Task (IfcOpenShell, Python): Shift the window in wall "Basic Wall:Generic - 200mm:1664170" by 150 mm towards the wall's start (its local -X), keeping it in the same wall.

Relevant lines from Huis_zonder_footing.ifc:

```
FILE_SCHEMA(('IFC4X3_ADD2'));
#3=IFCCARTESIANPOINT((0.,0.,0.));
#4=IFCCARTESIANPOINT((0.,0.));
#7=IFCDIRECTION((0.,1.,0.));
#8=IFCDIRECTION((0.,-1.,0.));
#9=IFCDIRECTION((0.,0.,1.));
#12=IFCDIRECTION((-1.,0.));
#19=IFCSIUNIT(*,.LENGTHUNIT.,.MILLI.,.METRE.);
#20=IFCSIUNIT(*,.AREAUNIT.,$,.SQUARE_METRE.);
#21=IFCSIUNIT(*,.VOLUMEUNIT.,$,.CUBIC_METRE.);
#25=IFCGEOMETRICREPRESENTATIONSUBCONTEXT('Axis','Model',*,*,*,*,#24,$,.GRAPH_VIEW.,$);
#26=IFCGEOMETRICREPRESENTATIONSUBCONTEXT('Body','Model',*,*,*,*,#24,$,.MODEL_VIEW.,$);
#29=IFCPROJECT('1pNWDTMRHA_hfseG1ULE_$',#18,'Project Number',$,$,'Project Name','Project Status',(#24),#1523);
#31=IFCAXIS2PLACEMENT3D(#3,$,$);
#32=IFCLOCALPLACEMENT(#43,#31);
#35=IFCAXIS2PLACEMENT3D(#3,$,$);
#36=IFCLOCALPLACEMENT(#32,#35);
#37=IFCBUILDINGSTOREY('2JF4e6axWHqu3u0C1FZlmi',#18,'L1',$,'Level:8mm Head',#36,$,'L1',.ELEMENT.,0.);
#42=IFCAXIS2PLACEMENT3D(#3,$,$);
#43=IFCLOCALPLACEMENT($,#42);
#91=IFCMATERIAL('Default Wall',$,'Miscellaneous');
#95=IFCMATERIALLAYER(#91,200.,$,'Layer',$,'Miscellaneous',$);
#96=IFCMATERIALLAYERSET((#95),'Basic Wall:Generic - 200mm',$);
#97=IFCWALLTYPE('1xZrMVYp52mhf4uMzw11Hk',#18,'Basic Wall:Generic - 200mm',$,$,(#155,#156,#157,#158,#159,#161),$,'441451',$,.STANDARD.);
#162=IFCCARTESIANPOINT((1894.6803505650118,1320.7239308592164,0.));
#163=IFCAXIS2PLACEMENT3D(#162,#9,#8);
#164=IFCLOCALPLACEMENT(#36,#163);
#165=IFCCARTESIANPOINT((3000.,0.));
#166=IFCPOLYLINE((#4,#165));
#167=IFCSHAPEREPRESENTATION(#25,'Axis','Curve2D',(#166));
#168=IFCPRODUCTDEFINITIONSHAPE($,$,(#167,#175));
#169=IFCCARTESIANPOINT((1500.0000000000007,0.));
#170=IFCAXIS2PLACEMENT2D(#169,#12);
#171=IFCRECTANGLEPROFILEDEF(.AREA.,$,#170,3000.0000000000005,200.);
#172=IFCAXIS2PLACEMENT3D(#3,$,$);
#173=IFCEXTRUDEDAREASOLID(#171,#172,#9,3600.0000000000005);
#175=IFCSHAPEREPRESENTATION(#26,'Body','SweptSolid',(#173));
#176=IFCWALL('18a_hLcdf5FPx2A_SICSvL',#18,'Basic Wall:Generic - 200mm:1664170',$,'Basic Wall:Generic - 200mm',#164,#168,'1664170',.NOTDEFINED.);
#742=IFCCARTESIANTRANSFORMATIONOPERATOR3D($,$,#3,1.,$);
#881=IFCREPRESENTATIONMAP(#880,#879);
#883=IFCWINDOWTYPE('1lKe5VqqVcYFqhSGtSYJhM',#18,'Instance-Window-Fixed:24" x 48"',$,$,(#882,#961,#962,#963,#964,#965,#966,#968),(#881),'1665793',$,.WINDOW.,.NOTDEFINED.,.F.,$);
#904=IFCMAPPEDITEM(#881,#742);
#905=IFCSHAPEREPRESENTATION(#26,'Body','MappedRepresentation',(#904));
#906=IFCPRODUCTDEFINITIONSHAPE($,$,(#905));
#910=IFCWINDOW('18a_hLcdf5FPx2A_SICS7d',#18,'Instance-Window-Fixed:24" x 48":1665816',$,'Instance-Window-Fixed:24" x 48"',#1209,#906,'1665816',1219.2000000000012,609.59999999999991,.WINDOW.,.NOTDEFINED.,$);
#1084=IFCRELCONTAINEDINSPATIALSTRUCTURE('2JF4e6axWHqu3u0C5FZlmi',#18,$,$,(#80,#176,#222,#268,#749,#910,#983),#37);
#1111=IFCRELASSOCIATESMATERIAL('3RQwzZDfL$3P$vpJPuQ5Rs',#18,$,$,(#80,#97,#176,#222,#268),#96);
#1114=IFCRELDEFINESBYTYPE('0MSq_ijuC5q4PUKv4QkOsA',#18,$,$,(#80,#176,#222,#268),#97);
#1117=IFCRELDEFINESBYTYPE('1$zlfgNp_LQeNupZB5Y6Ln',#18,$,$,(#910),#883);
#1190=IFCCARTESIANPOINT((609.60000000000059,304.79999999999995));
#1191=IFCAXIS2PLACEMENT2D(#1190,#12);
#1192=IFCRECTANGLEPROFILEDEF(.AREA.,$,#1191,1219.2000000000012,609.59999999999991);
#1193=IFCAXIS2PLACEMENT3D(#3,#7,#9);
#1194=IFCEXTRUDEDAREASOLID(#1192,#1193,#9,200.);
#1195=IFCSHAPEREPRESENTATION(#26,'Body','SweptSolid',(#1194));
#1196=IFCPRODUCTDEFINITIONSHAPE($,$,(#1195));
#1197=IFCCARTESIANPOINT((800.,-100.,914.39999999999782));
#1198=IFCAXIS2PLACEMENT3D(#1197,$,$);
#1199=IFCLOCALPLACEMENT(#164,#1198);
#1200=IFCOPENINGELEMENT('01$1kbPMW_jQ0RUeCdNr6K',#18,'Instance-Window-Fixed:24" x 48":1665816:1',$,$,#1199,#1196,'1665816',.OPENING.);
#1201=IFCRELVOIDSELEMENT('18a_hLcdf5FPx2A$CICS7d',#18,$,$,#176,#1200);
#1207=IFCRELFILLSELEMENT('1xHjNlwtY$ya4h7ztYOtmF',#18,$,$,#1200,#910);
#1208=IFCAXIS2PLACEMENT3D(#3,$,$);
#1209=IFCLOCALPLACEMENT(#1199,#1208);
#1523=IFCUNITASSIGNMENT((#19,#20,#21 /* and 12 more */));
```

```python
import ifcopenshell
import ifcopenshell.api.geometry
import ifcopenshell.util.placement

model = ifcopenshell.open("Huis_zonder_footing.ifc")

window = model.by_id(910)
opening = window.FillsVoids[0].RelatingOpeningElement
wall = opening.VoidsElements[0].RelatingBuildingElement

wall_matrix = ifcopenshell.util.placement.get_local_placement(wall.ObjectPlacement)
shift = wall_matrix[:3, 0] * -150.0
before = ifcopenshell.util.placement.get_local_placement(window.ObjectPlacement)[:3, 3].copy()

# The window is placed relative to its opening, so it follows when the opening moves.
matrix = ifcopenshell.util.placement.get_local_placement(opening.ObjectPlacement)
matrix[:3, 3] += shift
ifcopenshell.api.geometry.edit_object_placement(
    model, product=opening, matrix=matrix, is_si=False, should_transform_children=True
)

after = ifcopenshell.util.placement.get_local_placement(window.ObjectPlacement)[:3, 3]
print("window moved by", (after - before).round(3) + 0.0)

model.write("Huis_zonder_footing-out.ifc")
```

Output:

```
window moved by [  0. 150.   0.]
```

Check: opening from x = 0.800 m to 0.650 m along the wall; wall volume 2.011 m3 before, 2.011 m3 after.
